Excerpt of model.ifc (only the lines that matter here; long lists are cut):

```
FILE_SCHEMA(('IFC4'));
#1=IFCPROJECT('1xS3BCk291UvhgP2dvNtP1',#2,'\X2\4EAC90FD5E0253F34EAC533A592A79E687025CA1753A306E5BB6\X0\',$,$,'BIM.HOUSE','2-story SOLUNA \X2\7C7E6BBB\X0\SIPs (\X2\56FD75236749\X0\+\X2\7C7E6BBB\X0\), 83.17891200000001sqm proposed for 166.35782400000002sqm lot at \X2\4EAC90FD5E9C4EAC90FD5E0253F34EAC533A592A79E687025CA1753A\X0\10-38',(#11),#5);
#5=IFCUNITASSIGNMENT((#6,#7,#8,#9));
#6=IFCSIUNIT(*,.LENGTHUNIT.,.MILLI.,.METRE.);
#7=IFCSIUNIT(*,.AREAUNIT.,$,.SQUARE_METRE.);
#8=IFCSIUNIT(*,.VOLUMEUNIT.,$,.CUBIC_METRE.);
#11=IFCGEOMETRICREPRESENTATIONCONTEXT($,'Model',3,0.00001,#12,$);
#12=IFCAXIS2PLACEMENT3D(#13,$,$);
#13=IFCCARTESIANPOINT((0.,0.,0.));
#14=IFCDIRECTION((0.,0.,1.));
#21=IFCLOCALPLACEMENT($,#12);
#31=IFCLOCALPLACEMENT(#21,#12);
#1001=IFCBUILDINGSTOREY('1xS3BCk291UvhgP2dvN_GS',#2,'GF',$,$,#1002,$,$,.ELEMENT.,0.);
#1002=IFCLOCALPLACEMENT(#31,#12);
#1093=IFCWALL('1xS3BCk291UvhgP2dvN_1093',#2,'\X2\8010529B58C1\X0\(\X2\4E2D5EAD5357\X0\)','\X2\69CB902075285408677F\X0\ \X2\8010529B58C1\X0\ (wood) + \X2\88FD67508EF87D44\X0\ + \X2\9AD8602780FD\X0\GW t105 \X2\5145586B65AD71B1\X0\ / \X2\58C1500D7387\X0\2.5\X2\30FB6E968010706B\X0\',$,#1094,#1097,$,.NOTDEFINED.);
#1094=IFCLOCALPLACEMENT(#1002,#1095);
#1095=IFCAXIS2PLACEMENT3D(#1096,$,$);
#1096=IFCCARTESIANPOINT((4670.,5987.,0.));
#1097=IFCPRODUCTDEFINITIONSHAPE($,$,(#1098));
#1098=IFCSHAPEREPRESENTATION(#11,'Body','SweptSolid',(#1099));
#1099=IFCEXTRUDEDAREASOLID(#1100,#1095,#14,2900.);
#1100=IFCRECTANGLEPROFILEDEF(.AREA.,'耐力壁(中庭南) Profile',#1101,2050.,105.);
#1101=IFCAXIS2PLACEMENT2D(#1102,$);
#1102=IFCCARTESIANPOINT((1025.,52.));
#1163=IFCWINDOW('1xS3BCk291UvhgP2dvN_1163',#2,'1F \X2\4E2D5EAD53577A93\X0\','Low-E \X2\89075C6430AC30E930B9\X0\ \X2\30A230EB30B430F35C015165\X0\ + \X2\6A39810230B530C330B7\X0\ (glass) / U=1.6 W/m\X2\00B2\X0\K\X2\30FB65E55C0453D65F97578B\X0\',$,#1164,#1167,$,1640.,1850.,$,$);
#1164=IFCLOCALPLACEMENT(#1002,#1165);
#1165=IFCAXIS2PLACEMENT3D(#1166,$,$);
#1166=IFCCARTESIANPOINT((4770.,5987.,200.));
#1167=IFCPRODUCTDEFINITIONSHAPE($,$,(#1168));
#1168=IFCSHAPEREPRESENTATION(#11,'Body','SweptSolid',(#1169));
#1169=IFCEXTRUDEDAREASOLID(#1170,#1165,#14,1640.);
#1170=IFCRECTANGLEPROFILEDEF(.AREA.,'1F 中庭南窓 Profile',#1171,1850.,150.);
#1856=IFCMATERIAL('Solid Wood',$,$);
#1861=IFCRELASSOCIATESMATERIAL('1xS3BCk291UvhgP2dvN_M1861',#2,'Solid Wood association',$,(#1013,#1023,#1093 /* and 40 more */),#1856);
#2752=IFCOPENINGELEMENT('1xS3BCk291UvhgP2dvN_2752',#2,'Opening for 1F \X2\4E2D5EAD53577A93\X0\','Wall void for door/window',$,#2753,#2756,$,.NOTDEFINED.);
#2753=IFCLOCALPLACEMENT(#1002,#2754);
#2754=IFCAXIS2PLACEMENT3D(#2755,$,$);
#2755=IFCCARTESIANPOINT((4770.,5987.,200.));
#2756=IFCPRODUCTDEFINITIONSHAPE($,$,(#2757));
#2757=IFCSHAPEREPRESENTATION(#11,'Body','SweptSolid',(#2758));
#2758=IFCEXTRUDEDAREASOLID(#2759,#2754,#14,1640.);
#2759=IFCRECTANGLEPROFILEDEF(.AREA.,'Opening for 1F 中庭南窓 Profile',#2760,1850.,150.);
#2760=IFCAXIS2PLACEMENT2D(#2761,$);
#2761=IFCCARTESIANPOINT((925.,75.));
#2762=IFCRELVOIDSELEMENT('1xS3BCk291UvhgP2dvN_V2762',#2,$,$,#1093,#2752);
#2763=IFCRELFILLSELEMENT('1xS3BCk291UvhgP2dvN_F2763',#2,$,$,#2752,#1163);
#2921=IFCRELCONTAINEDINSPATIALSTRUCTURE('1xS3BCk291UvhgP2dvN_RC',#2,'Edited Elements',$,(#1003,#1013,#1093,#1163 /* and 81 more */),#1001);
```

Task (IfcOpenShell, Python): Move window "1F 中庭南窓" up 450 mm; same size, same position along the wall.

```python
import numpy as np
import ifcopenshell
import ifcopenshell.api.geometry
import ifcopenshell.util.placement
import ifcopenshell.util.unit

model = ifcopenshell.open("model.ifc")
unit_scale = ifcopenshell.util.unit.calculate_unit_scale(model)

window = model.by_guid("1xS3BCk291UvhgP2dvN_1163")
opening = window.FillsVoids[0].RelatingOpeningElement
dz = 0.45 / unit_scale

shift = np.array([0.0, 0.0, dz])
# The window is not placed relative to its opening, so move both.
for product in (opening, window):
    matrix = ifcopenshell.util.placement.get_local_placement(product.ObjectPlacement)
    matrix[:3, 3] += shift
    ifcopenshell.api.geometry.edit_object_placement(model, product=product, matrix=matrix, is_si=False)

print(f"moved by {dz * unit_scale:+.3f} m")

model.write("model_rev.ifc")
```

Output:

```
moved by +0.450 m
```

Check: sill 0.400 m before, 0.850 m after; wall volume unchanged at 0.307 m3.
